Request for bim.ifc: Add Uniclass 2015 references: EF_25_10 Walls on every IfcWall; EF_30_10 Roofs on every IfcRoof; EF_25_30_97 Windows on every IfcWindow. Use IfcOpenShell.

First a look at what the model holds.

```python
import ifcopenshell

model = ifcopenshell.open("bim.ifc")
print(model.schema)
print("classifications:", [c.Name for c in model.by_type("IfcClassification")])
for ifc_class in ("IfcDoor", "IfcRoof", "IfcStair", "IfcWall", "IfcWindow"):
    print(ifc_class, len(model.by_type(ifc_class)))
```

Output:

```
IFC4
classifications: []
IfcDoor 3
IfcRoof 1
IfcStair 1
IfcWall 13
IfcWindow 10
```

```python
import ifcopenshell
import ifcopenshell.api.classification

model = ifcopenshell.open("bim.ifc")

system = ifcopenshell.api.classification.add_classification(model, classification="Uniclass 2015")

codes = {
    "IfcWall": ("EF_25_10", "Walls"),
    "IfcRoof": ("EF_30_10", "Roofs"),
    "IfcWindow": ("EF_25_30_97", "Windows"),
}
for ifc_class, (code, name) in codes.items():
    products = model.by_type(ifc_class)
    ifcopenshell.api.classification.add_reference(
        model, products=products, classification=system, identification=code, name=name
    )
    print(code, len(products))

model.write("bim_edited.ifc")
```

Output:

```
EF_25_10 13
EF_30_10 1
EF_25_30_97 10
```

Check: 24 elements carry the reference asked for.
